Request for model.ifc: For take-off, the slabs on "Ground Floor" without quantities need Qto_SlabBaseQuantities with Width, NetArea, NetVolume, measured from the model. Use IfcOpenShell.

First a look at what the model holds.

```python
import ifcopenshell
import ifcopenshell.util.element
import ifcopenshell.util.unit

model = ifcopenshell.open("model.ifc")
print(model.schema)
for unit_type in ("LENGTHUNIT", "AREAUNIT", "VOLUMEUNIT"):
    print(unit_type, ifcopenshell.util.unit.calculate_unit_scale(model, unit_type))
storey = next(s for s in model.by_type("IfcBuildingStorey") if s.Name == "Ground Floor")
slabs = [e for e in ifcopenshell.util.element.get_decomposition(storey) if e.is_a("IfcSlab")]
for e in sorted(slabs, key=lambda e: e.id()):
    print(e.id(), e.is_a(), e.Name, list(ifcopenshell.util.element.get_psets(e, qtos_only=True)), sep=" | ")
```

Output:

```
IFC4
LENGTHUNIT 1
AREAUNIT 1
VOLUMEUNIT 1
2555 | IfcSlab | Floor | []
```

```python
import ifcopenshell
import ifcopenshell.api.pset
import ifcopenshell.geom
import ifcopenshell.util.element
import ifcopenshell.util.shape
import ifcopenshell.util.unit

model = ifcopenshell.open("model.ifc")
unit_scale = ifcopenshell.util.unit.calculate_unit_scale(model)
area_scale = ifcopenshell.util.unit.calculate_unit_scale(model, "AREAUNIT")
volume_scale = ifcopenshell.util.unit.calculate_unit_scale(model, "VOLUMEUNIT")
settings = ifcopenshell.geom.settings()

storey = next(s for s in model.by_type("IfcBuildingStorey") if s.Name == "Ground Floor")
slabs = [e for e in ifcopenshell.util.element.get_decomposition(storey) if e.is_a("IfcSlab")]

for e in sorted(slabs, key=lambda e: e.id()):
    if ifcopenshell.util.element.get_psets(e, qtos_only=True, should_inherit=False):
        continue
    # Geometry comes back in metres, in the element's own axes.
    shape = ifcopenshell.geom.create_shape(settings, e)
    values = {
        "Width": ifcopenshell.util.shape.get_z(shape.geometry) / unit_scale,
        "NetArea": ifcopenshell.util.shape.get_footprint_area(shape.geometry) / area_scale,
        "NetVolume": ifcopenshell.util.shape.get_volume(shape.geometry) / volume_scale,
    }
    qto = ifcopenshell.api.pset.add_qto(model, product=e, name="Qto_SlabBaseQuantities")
    ifcopenshell.api.pset.edit_qto(model, qto=qto, properties=values)
    print(e.id(), {k: round(v, 3) for k, v in values.items()})

model.write("model_v2.ifc")
```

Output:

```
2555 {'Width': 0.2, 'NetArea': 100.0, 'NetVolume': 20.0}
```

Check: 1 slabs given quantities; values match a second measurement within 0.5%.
